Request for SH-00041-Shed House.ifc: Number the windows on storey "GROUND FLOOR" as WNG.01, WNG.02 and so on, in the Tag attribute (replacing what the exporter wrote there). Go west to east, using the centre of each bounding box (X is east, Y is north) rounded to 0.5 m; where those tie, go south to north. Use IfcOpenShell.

First a look at what the model holds.

```python
import ifcopenshell
import ifcopenshell.util.element
import ifcopenshell.util.placement

model = ifcopenshell.open("SH-00041-Shed House.ifc")
print(model.schema)
storey = next(s for s in model.by_type("IfcBuildingStorey") if s.Name == "GROUND FLOOR")
windows = [e for e in ifcopenshell.util.element.get_decomposition(storey) if e.is_a("IfcWindow")]
for e in sorted(windows, key=lambda e: e.id()):
    origin = ifcopenshell.util.placement.get_local_placement(e.ObjectPlacement)[:3, 3]
    print(e.id(), e.Tag, e.Name, origin.round(2) + 0.0, sep=" | ")
```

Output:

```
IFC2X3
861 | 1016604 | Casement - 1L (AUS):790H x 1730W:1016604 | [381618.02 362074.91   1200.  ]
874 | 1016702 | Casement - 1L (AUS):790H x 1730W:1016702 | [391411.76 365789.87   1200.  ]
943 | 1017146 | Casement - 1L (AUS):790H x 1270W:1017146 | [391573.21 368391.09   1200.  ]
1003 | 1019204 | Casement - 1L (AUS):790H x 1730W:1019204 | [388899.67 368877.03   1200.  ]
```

```python
import ifcopenshell
import ifcopenshell.geom
import ifcopenshell.util.element
import ifcopenshell.util.shape

model = ifcopenshell.open("SH-00041-Shed House.ifc")
settings = ifcopenshell.geom.settings()
settings.set("use-world-coords", True)


def centre(element):
    shape = ifcopenshell.geom.create_shape(settings, element)
    return ifcopenshell.util.shape.get_bbox_centroid(shape.geometry)


storey = next(s for s in model.by_type("IfcBuildingStorey") if s.Name == "GROUND FLOOR")
windows = [e for e in ifcopenshell.util.element.get_decomposition(storey) if e.is_a("IfcWindow")]

# Insertion points can sit at a corner or the storey origin, so sort by the geometry (in metres).
centres = {e: centre(e) for e in windows}
windows.sort(key=lambda e: (round(centres[e][0] / 0.5), centres[e][1]))

for i, e in enumerate(windows, start=1):
    number = f"WNG.{i:02d}"
    e.Tag = number
    print(e.id(), number)

model.write("SH-00041-Shed House_edited.ifc")
```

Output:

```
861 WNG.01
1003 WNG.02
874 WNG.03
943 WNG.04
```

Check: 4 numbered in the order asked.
